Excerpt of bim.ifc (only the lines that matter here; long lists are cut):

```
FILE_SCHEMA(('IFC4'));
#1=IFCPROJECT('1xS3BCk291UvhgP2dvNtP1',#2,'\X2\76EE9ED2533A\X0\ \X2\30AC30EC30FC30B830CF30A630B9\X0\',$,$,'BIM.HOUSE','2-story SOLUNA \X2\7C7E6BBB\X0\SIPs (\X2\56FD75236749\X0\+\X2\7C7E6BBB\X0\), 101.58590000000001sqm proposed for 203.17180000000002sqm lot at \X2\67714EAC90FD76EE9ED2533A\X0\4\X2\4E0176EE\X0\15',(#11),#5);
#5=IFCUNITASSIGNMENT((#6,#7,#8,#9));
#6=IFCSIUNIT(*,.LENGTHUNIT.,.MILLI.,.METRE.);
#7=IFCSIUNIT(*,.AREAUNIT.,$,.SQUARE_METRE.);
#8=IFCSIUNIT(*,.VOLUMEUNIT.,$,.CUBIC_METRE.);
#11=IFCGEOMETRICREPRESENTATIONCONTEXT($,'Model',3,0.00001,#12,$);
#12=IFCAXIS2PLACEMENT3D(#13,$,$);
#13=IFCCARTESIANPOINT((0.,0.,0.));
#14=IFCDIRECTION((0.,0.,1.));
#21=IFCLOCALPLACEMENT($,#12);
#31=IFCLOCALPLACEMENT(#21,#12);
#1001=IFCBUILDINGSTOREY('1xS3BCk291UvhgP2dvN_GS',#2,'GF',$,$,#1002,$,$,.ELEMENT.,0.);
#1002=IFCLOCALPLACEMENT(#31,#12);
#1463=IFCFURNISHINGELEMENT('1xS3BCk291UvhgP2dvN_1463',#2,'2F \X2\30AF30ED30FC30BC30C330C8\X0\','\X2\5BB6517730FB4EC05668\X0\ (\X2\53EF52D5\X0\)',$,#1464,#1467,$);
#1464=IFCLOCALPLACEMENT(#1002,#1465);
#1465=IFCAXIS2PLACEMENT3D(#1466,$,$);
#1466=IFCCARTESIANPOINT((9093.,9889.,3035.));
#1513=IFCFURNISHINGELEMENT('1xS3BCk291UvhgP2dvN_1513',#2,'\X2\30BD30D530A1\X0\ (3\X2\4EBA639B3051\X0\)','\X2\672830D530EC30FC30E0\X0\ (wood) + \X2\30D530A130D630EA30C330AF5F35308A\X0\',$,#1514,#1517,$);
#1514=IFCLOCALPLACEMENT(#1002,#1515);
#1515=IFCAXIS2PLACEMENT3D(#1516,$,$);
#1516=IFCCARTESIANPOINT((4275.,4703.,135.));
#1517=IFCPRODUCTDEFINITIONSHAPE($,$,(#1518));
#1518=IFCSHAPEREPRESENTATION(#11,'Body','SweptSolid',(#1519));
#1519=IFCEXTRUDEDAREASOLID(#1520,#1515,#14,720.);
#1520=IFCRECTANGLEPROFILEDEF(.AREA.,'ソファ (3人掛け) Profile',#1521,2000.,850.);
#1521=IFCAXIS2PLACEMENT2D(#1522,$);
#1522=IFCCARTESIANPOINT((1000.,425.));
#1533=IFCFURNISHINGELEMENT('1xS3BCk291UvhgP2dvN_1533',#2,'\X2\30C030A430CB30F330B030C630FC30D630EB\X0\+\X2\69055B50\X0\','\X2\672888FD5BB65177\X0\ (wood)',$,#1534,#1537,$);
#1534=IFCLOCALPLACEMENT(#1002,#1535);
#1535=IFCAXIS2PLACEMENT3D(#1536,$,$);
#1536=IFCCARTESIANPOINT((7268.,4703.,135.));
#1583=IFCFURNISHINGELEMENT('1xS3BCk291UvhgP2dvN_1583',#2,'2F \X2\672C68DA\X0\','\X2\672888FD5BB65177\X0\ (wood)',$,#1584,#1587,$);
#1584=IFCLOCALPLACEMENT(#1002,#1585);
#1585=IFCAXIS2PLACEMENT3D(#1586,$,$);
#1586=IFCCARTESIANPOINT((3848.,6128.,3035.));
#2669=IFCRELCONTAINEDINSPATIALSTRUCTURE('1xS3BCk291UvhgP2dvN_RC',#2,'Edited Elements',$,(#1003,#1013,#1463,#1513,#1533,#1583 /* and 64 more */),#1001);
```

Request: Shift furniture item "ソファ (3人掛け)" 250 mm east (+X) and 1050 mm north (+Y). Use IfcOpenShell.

```python
import ifcopenshell
import ifcopenshell.api.geometry
import ifcopenshell.util.placement

model = ifcopenshell.open("bim.ifc")

item = model.by_guid("1xS3BCk291UvhgP2dvN_1513")
matrix = ifcopenshell.util.placement.get_local_placement(item.ObjectPlacement)
matrix[0, 3] += 250.0
matrix[1, 3] += 1050.0
ifcopenshell.api.geometry.edit_object_placement(model, product=item, matrix=matrix, is_si=False)

print(ifcopenshell.util.placement.get_local_placement(item.ObjectPlacement).round(3) + 0.0)

model.write("bim-out.ifc")
```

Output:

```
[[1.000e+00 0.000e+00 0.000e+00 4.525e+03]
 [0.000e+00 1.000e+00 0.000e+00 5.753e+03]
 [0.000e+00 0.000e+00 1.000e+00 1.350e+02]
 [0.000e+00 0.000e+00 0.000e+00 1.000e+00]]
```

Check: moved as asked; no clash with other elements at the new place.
